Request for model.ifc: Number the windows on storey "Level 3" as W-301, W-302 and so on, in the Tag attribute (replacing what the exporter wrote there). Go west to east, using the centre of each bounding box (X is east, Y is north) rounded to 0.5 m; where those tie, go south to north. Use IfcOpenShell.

First a look at what the model holds.

```python
import ifcopenshell
import ifcopenshell.util.element
import ifcopenshell.util.placement

model = ifcopenshell.open("model.ifc")
print(model.schema)
storey = next(s for s in model.by_type("IfcBuildingStorey") if s.Name == "Level 3")
windows = [e for e in ifcopenshell.util.element.get_decomposition(storey) if e.is_a("IfcWindow")]
for e in sorted(windows, key=lambda e: e.id()):
    origin = ifcopenshell.util.placement.get_local_placement(e.ObjectPlacement)[:3, 3]
    print(e.id(), e.Tag, e.Name, origin.round(2) + 0.0, sep=" | ")
```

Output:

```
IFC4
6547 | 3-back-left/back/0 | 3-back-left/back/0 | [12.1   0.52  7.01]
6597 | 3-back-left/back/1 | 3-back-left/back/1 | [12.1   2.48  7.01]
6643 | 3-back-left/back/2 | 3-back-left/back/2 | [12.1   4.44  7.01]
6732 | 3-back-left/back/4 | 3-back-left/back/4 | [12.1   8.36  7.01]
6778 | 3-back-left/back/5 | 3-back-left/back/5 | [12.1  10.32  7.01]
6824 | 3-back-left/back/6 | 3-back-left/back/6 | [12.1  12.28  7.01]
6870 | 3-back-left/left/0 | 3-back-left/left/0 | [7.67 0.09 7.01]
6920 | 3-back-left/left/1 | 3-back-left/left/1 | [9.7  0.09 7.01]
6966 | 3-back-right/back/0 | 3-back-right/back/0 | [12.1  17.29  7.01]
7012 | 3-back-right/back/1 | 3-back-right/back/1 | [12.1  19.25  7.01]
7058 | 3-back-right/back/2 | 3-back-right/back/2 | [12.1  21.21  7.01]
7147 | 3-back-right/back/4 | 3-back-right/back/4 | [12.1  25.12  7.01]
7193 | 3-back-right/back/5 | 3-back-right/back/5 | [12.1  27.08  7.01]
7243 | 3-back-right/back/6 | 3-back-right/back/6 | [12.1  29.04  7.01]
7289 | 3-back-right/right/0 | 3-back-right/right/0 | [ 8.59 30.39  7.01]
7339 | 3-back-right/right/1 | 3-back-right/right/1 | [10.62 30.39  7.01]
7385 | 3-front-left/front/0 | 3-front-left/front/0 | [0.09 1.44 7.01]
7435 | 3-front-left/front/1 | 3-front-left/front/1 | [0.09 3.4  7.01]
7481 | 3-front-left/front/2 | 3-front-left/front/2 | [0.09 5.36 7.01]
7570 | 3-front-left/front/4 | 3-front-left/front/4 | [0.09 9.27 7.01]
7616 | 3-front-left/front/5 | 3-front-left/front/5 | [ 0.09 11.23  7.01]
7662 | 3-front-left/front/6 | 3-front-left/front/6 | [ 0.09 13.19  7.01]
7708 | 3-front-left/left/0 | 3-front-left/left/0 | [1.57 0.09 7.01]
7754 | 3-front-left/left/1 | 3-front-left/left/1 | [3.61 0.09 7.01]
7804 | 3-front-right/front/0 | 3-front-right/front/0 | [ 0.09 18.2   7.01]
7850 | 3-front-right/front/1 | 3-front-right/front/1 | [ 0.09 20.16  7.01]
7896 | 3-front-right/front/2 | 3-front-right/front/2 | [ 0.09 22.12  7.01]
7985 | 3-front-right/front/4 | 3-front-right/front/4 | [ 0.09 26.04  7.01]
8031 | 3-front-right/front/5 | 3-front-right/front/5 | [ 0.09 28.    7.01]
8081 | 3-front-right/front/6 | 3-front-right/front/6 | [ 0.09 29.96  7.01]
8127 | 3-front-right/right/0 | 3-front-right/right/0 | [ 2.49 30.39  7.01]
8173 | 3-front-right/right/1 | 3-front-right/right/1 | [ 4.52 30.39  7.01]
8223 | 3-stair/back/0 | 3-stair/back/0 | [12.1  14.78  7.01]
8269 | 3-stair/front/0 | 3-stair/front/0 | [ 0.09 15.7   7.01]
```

```python
import ifcopenshell
import ifcopenshell.geom
import ifcopenshell.util.element
import ifcopenshell.util.shape

model = ifcopenshell.open("model.ifc")
settings = ifcopenshell.geom.settings()
settings.set("use-world-coords", True)


def centre(element):
    shape = ifcopenshell.geom.create_shape(settings, element)
    return ifcopenshell.util.shape.get_bbox_centroid(shape.geometry)


storey = next(s for s in model.by_type("IfcBuildingStorey") if s.Name == "Level 3")
windows = [e for e in ifcopenshell.util.element.get_decomposition(storey) if e.is_a("IfcWindow")]

# Insertion points can sit at a corner or the storey origin, so sort by the geometry (in metres).
centres = {e: centre(e) for e in windows}
windows.sort(key=lambda e: (round(centres[e][0] / 0.5), centres[e][1]))

for i, e in enumerate(windows, start=1):
    number = f"W-3{i:02d}"
    e.Tag = number
    print(e.id(), number)

model.write("model_updated.ifc")
```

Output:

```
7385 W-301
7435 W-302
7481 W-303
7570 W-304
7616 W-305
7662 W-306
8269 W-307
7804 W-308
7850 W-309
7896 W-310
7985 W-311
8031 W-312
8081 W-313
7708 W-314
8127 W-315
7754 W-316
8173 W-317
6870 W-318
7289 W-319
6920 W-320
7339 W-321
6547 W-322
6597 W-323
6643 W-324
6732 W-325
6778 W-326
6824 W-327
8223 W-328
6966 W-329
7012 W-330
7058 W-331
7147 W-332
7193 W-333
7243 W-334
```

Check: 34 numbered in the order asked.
